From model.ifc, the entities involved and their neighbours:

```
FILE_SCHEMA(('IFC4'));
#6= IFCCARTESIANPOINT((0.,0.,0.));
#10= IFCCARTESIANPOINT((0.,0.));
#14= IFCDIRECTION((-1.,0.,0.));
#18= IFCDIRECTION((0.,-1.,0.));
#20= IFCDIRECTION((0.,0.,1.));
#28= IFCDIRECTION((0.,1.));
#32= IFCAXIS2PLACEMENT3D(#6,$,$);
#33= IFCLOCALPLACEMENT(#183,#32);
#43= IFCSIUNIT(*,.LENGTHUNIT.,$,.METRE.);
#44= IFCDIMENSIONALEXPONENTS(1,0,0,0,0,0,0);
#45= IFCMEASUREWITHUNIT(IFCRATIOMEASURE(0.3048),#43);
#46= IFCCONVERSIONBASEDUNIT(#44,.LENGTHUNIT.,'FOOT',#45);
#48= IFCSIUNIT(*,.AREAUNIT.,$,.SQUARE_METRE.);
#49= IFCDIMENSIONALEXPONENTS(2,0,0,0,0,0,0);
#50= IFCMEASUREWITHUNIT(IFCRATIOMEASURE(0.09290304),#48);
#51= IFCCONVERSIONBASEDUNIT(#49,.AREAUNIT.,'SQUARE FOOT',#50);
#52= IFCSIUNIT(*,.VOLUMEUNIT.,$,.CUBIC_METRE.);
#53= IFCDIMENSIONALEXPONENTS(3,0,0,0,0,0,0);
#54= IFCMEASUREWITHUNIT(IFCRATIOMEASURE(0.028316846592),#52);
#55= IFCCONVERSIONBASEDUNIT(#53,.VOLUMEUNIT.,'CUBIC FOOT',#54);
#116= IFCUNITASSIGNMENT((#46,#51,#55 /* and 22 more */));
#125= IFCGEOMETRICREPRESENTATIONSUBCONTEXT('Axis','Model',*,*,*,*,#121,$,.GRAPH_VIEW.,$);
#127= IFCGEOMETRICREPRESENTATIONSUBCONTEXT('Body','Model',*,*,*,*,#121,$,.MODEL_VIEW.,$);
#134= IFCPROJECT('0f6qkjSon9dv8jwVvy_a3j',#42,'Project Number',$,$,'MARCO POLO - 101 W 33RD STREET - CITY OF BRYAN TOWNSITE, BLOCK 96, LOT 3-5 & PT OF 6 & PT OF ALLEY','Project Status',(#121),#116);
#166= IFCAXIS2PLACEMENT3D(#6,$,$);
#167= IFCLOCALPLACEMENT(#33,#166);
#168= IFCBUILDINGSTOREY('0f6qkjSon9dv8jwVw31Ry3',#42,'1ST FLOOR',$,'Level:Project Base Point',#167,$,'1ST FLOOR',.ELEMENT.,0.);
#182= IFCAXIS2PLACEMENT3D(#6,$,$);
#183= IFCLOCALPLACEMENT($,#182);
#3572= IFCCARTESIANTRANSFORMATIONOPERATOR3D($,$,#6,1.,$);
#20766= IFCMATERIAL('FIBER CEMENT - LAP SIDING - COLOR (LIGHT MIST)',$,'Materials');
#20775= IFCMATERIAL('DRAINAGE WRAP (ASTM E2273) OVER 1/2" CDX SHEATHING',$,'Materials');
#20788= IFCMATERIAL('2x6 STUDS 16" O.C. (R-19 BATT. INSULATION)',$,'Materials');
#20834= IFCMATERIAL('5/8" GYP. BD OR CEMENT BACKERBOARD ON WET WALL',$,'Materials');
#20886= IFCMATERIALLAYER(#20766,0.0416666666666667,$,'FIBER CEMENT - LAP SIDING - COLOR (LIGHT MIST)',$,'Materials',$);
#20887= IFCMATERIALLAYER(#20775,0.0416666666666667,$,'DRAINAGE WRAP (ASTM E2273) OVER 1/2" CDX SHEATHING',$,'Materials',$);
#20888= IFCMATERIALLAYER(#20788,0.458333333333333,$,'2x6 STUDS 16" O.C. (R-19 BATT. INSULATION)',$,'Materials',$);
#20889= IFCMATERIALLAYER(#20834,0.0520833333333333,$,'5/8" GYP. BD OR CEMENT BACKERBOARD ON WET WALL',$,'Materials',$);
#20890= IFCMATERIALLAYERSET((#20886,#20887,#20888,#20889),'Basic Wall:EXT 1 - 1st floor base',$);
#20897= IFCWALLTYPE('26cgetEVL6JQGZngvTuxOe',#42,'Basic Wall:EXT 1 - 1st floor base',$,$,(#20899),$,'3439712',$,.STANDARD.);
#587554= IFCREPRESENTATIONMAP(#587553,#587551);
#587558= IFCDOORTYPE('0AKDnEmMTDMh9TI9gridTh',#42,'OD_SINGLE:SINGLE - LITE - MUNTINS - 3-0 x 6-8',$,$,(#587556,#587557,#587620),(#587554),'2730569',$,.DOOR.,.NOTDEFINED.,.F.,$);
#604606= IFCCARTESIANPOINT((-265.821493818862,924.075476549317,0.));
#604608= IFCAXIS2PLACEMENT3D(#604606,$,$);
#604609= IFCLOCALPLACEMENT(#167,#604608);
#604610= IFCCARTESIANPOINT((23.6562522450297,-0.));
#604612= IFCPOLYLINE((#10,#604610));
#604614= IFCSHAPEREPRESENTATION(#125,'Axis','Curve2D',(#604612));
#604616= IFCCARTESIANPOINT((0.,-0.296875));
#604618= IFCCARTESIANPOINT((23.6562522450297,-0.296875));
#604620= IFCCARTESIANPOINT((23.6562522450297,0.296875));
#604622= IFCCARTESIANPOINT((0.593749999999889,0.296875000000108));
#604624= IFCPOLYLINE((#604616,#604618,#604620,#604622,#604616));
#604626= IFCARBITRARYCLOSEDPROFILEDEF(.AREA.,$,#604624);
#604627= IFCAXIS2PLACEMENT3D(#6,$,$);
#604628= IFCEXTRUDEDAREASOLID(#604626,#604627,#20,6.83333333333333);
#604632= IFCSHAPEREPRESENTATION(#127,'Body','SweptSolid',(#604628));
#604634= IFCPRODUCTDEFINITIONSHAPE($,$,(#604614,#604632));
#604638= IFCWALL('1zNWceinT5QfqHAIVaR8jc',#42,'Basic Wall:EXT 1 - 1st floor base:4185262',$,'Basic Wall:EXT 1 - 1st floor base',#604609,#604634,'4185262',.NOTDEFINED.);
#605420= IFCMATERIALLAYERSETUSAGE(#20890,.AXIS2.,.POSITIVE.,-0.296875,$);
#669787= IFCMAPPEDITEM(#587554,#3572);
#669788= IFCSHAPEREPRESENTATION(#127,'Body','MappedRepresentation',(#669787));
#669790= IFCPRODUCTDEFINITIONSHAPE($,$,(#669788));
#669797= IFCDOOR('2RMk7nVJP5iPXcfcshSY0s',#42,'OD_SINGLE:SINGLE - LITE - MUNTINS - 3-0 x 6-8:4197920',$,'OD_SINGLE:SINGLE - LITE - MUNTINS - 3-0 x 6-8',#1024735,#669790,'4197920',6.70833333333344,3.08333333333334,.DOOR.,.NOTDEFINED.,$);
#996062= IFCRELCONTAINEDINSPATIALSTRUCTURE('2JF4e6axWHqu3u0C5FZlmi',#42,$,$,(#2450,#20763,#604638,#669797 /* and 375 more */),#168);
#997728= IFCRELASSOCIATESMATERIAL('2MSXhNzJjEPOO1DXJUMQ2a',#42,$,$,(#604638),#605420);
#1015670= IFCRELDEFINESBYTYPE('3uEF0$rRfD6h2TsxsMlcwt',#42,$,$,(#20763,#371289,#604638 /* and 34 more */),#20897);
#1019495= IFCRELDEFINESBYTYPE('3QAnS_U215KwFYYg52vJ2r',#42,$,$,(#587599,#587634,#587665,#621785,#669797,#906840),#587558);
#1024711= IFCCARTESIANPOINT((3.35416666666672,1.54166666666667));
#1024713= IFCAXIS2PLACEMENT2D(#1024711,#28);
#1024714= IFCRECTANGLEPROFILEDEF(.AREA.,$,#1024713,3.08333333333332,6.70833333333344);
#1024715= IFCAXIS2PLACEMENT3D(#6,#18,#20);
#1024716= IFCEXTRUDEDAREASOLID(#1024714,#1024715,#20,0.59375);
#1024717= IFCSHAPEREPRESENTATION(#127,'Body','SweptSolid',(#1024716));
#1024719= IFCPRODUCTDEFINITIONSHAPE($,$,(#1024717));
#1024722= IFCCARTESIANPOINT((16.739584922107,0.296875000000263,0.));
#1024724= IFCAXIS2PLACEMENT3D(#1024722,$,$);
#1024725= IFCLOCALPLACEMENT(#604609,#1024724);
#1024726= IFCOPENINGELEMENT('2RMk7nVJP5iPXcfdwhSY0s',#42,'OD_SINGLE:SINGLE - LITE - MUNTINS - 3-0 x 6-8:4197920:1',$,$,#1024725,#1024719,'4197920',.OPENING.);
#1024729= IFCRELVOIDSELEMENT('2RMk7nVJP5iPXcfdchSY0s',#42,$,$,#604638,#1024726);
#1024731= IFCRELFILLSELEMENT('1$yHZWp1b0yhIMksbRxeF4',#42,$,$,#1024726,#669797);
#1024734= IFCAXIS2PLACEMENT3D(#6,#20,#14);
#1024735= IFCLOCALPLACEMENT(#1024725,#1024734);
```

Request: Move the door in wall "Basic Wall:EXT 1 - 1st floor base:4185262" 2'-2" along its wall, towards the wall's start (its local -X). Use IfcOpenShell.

```python
import ifcopenshell
import ifcopenshell.api.geometry
import ifcopenshell.util.placement
import ifcopenshell.util.unit

model = ifcopenshell.open("model.ifc")
unit_scale = ifcopenshell.util.unit.calculate_unit_scale(model)

door = model.by_id(669797)
opening = door.FillsVoids[0].RelatingOpeningElement
wall = opening.VoidsElements[0].RelatingBuildingElement

wall_matrix = ifcopenshell.util.placement.get_local_placement(wall.ObjectPlacement)
shift = wall_matrix[:3, 0] * -26 * 0.0254 / unit_scale
before = ifcopenshell.util.placement.get_local_placement(door.ObjectPlacement)[:3, 3].copy()

# The door is placed relative to its opening, so it follows when the opening moves.
matrix = ifcopenshell.util.placement.get_local_placement(opening.ObjectPlacement)
matrix[:3, 3] += shift
ifcopenshell.api.geometry.edit_object_placement(
    model, product=opening, matrix=matrix, is_si=False, should_transform_children=True
)

after = ifcopenshell.util.placement.get_local_placement(door.ObjectPlacement)[:3, 3]
print("door moved by", (after - before).round(3) + 0.0)

model.write("model_v2.ifc")
```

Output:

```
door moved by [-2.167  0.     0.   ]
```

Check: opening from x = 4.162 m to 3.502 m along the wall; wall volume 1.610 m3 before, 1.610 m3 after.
